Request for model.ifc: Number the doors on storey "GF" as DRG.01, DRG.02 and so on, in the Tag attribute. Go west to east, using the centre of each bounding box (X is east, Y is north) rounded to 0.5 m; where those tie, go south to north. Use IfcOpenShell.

First a look at what the model holds.

```python
import ifcopenshell
import ifcopenshell.util.element
import ifcopenshell.util.placement

model = ifcopenshell.open("model.ifc")
print(model.schema)
storey = next(s for s in model.by_type("IfcBuildingStorey") if s.Name == "GF")
doors = [e for e in ifcopenshell.util.element.get_decomposition(storey) if e.is_a("IfcDoor")]
for e in sorted(doors, key=lambda e: e.id()):
    origin = ifcopenshell.util.placement.get_local_placement(e.ObjectPlacement)[:3, 3]
    print(e.id(), e.Tag, e.Name, origin.round(2) + 0.0, sep=" | ")
```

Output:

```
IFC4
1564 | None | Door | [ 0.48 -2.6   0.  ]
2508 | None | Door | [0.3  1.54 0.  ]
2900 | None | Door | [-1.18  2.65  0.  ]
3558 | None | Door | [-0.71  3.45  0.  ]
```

```python
import ifcopenshell
import ifcopenshell.geom
import ifcopenshell.util.element
import ifcopenshell.util.shape

model = ifcopenshell.open("model.ifc")
settings = ifcopenshell.geom.settings()
settings.set("use-world-coords", True)


def centre(element):
    shape = ifcopenshell.geom.create_shape(settings, element)
    return ifcopenshell.util.shape.get_bbox_centroid(shape.geometry)


storey = next(s for s in model.by_type("IfcBuildingStorey") if s.Name == "GF")
doors = [e for e in ifcopenshell.util.element.get_decomposition(storey) if e.is_a("IfcDoor")]

# Insertion points can sit at a corner or the storey origin, so sort by the geometry (in metres).
centres = {e: centre(e) for e in doors}
doors.sort(key=lambda e: (round(centres[e][0] / 0.5), centres[e][1]))

for i, e in enumerate(doors, start=1):
    number = f"DRG.{i:02d}"
    e.Tag = number
    print(e.id(), number)

model.write("model_edited.ifc")
```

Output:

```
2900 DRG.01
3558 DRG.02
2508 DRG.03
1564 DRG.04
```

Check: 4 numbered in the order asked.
